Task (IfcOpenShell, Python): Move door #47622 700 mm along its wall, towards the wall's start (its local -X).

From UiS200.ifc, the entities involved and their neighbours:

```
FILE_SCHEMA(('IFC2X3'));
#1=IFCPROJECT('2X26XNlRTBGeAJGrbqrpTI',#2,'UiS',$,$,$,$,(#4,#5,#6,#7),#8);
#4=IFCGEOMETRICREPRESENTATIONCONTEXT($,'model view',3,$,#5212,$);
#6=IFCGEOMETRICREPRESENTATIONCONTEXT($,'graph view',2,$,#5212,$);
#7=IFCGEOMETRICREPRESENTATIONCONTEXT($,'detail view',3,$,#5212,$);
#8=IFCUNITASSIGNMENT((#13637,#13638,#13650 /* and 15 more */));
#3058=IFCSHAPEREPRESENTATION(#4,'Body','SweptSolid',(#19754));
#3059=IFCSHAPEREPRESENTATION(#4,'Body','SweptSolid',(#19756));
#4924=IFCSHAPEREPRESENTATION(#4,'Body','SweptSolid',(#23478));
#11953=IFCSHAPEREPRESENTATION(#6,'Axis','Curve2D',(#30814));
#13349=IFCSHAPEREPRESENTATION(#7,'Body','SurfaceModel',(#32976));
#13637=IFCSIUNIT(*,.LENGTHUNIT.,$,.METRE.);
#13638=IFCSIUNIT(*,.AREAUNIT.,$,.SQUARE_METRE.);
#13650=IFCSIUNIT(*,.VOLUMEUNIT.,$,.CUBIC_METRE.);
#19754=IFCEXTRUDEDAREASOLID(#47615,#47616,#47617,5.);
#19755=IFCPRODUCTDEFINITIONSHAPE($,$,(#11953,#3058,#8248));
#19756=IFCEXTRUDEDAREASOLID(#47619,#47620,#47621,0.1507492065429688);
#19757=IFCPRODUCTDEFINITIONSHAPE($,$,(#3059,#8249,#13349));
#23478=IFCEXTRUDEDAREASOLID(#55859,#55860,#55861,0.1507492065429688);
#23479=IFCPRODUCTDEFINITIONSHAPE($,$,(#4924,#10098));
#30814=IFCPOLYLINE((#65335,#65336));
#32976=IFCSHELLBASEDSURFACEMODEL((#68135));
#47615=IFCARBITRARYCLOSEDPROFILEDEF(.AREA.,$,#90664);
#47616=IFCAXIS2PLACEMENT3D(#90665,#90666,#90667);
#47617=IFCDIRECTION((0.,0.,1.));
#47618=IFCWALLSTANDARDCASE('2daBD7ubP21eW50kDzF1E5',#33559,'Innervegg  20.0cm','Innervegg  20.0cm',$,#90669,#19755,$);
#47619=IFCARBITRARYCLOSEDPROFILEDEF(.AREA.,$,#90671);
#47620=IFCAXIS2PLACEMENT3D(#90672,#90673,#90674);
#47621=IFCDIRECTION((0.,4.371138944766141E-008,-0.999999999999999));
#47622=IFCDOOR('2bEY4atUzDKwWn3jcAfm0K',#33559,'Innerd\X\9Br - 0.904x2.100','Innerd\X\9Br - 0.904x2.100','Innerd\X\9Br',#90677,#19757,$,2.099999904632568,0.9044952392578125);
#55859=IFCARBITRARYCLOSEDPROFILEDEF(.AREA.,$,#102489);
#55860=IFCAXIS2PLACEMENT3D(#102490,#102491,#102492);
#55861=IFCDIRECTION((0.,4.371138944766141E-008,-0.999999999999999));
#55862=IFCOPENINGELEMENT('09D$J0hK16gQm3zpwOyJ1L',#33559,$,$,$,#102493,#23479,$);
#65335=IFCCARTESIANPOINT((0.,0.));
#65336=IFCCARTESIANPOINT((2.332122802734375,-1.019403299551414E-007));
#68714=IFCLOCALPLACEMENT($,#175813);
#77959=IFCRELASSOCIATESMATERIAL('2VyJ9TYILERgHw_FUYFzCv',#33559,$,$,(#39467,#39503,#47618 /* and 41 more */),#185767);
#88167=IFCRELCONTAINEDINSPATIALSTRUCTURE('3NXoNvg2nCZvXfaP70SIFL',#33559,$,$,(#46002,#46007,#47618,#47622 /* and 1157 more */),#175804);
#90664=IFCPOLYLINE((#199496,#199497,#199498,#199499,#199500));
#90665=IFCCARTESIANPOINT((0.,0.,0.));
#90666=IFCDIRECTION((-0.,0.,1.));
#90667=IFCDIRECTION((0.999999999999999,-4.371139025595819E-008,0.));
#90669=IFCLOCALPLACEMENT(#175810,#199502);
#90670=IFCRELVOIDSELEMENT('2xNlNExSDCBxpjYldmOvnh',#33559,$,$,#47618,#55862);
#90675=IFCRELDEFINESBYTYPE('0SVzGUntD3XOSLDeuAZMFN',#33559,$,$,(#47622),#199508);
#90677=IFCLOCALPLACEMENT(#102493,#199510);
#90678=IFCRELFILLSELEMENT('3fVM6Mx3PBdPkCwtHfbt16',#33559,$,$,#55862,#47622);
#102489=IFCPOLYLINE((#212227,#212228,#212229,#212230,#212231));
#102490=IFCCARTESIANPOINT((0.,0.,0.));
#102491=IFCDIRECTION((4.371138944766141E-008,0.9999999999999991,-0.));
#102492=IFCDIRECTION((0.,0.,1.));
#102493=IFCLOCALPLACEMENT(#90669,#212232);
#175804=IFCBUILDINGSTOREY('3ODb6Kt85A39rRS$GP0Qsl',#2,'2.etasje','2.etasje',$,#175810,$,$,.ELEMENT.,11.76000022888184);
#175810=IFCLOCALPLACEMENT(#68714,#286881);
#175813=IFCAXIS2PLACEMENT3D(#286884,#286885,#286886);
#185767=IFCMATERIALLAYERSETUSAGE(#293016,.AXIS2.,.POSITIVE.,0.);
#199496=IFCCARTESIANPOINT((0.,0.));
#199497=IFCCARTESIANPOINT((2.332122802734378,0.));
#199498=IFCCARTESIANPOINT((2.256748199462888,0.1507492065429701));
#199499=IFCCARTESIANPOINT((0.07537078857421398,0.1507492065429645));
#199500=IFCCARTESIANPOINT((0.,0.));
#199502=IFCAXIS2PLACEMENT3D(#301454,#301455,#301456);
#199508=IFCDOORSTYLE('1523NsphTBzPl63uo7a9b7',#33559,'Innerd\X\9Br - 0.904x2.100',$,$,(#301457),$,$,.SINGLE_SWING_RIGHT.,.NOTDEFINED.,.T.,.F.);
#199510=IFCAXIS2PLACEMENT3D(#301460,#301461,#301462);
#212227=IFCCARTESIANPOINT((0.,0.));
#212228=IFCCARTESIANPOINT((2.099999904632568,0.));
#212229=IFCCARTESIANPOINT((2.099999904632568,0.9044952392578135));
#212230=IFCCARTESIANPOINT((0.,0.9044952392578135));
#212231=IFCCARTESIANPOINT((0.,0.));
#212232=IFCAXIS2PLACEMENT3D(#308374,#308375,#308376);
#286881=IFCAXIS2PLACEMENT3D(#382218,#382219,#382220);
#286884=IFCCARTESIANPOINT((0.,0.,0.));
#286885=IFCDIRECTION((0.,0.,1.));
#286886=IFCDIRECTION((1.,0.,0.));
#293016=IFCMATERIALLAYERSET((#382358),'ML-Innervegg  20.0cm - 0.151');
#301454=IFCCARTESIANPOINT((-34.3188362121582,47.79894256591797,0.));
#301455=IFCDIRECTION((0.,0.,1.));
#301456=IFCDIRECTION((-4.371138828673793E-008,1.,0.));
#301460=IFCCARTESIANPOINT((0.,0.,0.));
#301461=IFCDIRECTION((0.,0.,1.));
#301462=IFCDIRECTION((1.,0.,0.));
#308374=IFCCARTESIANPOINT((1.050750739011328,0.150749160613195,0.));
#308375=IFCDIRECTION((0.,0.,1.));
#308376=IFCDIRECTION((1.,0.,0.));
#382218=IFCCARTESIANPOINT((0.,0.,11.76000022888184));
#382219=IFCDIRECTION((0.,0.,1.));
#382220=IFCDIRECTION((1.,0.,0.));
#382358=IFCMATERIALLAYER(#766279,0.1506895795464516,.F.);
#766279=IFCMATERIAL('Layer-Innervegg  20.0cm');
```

```python
import ifcopenshell
import ifcopenshell.api.geometry
import ifcopenshell.util.placement
import ifcopenshell.util.unit

model = ifcopenshell.open("UiS200.ifc")
unit_scale = ifcopenshell.util.unit.calculate_unit_scale(model)

door = model.by_guid("2bEY4atUzDKwWn3jcAfm0K")
opening = door.FillsVoids[0].RelatingOpeningElement
wall = opening.VoidsElements[0].RelatingBuildingElement

wall_matrix = ifcopenshell.util.placement.get_local_placement(wall.ObjectPlacement)
shift = wall_matrix[:3, 0] * -0.7 / unit_scale
before = ifcopenshell.util.placement.get_local_placement(door.ObjectPlacement)[:3, 3].copy()

# The door is placed relative to its opening, so it follows when the opening moves.
matrix = ifcopenshell.util.placement.get_local_placement(opening.ObjectPlacement)
matrix[:3, 3] += shift
ifcopenshell.api.geometry.edit_object_placement(
    model, product=opening, matrix=matrix, is_si=False, should_transform_children=True
)

after = ifcopenshell.util.placement.get_local_placement(door.ObjectPlacement)[:3, 3]
print("door moved by", (after - before).round(3) + 0.0)

model.write("UiS200_rev.ifc")
```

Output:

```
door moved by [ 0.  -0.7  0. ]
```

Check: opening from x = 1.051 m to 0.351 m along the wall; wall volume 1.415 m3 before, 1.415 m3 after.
